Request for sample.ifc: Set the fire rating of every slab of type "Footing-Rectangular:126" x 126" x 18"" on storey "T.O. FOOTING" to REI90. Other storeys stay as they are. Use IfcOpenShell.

First a look at what the model holds.

```python
import ifcopenshell
import ifcopenshell.util.element

model = ifcopenshell.open("sample.ifc")
print(model.schema)
storey = next(s for s in model.by_type("IfcBuildingStorey") if s.Name == "T.O. FOOTING")
slabs = [e for e in ifcopenshell.util.element.get_decomposition(storey) if e.is_a("IfcSlab")]
seen = {}
for e in slabs:
    element_type = ifcopenshell.util.element.get_type(e)
    key = (element_type.Name if element_type != e and element_type else None, ifcopenshell.util.element.get_pset(e, "Pset_SlabCommon", "FireRating"))
    seen[key] = seen.get(key, 0) + 1
for (name, value), count in sorted(seen.items(), key=str):
    print(count, "x", name, "|", value)
```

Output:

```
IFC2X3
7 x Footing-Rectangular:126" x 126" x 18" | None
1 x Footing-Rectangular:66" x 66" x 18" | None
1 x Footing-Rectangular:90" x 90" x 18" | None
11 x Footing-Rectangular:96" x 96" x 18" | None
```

```python
import ifcopenshell
import ifcopenshell.api.pset
import ifcopenshell.util.element

model = ifcopenshell.open("sample.ifc")

storey = next(s for s in model.by_type("IfcBuildingStorey") if s.Name == "T.O. FOOTING")
slabs = [e for e in ifcopenshell.util.element.get_decomposition(storey) if e.is_a("IfcSlab")]

count = 0
for e in slabs:
    element_type = ifcopenshell.util.element.get_type(e)
    if element_type in (None, e) or element_type.Name != 'Footing-Rectangular:126" x 126" x 18"':
        continue
    # add_pset returns the element's existing set when there is one.
    pset = ifcopenshell.api.pset.add_pset(model, product=e, name="Pset_SlabCommon")
    ifcopenshell.api.pset.edit_pset(model, pset=pset, properties={"FireRating": "REI90"})
    count += 1

print(count, "slabs updated")

model.write("sample_edited.ifc")
```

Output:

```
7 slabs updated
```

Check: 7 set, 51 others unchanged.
